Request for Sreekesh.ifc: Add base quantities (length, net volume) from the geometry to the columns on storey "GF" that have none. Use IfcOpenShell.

First a look at what the model holds.

```python
import ifcopenshell
import ifcopenshell.util.element
import ifcopenshell.util.unit

model = ifcopenshell.open("Sreekesh.ifc")
print(model.schema)
for unit_type in ("LENGTHUNIT", "AREAUNIT", "VOLUMEUNIT"):
    print(unit_type, ifcopenshell.util.unit.calculate_unit_scale(model, unit_type))
storey = next(s for s in model.by_type("IfcBuildingStorey") if s.Name == "GF")
columns = [e for e in ifcopenshell.util.element.get_decomposition(storey) if e.is_a("IfcColumn")]
for e in sorted(columns, key=lambda e: e.id()):
    print(e.id(), e.is_a(), e.Name, list(ifcopenshell.util.element.get_psets(e, qtos_only=True)), sep=" | ")
```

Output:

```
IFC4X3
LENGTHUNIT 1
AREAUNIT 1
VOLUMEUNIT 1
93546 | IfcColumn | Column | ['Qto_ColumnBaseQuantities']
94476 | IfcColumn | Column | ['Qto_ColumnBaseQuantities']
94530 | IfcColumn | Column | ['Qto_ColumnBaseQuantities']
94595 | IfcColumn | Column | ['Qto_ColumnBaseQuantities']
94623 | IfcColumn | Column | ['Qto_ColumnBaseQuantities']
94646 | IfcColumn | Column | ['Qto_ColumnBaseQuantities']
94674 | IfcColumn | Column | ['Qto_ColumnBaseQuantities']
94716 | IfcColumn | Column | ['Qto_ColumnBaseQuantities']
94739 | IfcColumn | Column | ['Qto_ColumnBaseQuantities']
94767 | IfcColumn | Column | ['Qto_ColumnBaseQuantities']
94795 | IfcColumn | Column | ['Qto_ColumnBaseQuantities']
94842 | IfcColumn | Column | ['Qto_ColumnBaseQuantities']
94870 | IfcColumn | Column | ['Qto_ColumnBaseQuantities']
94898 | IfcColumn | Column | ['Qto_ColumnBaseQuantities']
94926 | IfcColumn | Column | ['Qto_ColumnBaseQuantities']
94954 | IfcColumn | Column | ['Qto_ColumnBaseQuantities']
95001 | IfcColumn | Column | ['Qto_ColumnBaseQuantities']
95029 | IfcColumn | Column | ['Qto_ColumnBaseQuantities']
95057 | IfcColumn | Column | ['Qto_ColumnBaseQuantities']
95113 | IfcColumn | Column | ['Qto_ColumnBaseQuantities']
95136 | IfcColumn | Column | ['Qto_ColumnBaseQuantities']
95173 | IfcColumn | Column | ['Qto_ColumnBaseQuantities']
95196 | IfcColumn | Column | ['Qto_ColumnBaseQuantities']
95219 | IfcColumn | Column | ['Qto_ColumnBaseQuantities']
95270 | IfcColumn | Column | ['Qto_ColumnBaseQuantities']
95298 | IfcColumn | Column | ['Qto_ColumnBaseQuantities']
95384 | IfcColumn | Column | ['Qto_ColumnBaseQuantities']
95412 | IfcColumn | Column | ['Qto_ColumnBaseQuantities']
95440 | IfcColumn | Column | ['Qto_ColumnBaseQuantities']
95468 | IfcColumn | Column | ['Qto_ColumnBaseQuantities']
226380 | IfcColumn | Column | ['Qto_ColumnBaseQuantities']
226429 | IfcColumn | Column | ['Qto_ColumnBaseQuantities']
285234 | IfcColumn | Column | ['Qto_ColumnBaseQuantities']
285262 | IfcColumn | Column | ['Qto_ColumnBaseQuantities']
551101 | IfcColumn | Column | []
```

```python
import ifcopenshell
import ifcopenshell.api.pset
import ifcopenshell.geom
import ifcopenshell.util.element
import ifcopenshell.util.shape
import ifcopenshell.util.unit

model = ifcopenshell.open("Sreekesh.ifc")
unit_scale = ifcopenshell.util.unit.calculate_unit_scale(model)
volume_scale = ifcopenshell.util.unit.calculate_unit_scale(model, "VOLUMEUNIT")
settings = ifcopenshell.geom.settings()

storey = next(s for s in model.by_type("IfcBuildingStorey") if s.Name == "GF")
columns = [e for e in ifcopenshell.util.element.get_decomposition(storey) if e.is_a("IfcColumn")]

for e in sorted(columns, key=lambda e: e.id()):
    if ifcopenshell.util.element.get_psets(e, qtos_only=True, should_inherit=False):
        continue
    # Geometry comes back in metres, in the element's own axes.
    shape = ifcopenshell.geom.create_shape(settings, e)
    values = {
        "Length": ifcopenshell.util.shape.get_z(shape.geometry) / unit_scale,
        "NetVolume": ifcopenshell.util.shape.get_volume(shape.geometry) / volume_scale,
    }
    qto = ifcopenshell.api.pset.add_qto(model, product=e, name="Qto_ColumnBaseQuantities")
    ifcopenshell.api.pset.edit_qto(model, qto=qto, properties=values)
    print(e.id(), {k: round(v, 3) for k, v in values.items()})

model.write("Sreekesh-out.ifc")
```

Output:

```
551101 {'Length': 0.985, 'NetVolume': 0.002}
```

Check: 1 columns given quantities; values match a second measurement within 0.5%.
